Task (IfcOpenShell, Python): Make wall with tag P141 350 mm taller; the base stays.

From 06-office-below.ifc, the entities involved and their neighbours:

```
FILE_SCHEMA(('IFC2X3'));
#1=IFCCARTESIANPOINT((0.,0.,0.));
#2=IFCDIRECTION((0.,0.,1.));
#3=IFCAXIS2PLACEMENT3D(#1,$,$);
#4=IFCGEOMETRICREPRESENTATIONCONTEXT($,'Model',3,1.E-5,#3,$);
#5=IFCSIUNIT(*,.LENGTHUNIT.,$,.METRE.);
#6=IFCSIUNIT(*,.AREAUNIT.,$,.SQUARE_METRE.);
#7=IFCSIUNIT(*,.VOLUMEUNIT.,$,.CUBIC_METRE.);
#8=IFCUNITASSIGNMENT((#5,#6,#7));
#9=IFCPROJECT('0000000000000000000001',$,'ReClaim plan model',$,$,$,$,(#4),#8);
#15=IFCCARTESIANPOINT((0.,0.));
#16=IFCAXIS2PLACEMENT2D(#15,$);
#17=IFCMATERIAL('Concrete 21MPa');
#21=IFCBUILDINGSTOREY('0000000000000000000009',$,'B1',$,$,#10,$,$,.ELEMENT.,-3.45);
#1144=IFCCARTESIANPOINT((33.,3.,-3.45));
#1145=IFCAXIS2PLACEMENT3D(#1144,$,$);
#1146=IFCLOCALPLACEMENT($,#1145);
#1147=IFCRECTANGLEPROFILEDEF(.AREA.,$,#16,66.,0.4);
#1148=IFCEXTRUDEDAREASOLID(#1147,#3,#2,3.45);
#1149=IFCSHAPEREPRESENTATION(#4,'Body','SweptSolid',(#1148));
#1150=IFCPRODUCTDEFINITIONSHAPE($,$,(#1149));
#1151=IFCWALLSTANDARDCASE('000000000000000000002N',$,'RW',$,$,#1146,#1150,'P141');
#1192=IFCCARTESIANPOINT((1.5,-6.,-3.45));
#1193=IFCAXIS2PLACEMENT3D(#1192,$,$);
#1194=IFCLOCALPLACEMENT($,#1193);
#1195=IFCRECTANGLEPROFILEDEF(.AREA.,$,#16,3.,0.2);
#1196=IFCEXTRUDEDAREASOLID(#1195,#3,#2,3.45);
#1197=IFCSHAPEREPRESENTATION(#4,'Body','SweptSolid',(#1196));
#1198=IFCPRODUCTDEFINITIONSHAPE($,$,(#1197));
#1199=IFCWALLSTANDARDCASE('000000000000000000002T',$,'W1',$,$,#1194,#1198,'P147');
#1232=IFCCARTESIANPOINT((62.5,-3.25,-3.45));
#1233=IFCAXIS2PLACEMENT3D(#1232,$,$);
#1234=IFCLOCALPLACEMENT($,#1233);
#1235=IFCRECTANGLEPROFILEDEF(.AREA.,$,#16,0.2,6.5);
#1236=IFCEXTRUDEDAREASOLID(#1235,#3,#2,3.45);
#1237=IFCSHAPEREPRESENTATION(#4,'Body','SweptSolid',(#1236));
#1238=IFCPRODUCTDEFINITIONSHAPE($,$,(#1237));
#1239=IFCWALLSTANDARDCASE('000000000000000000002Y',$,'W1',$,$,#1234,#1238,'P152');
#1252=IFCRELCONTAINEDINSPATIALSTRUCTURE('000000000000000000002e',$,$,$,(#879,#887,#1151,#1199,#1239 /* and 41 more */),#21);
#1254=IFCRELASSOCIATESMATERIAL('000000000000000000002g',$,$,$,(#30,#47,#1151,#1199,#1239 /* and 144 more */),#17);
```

```python
import ifcopenshell
import ifcopenshell.geom
import ifcopenshell.util.shape

model = ifcopenshell.open("06-office-below.ifc")
settings = ifcopenshell.geom.settings()


def volume(element):
    """Net volume in cubic metres, openings subtracted."""
    shape = ifcopenshell.geom.create_shape(settings, element)
    return ifcopenshell.util.shape.get_volume(shape.geometry)


wall = model.by_id(1151)
before = volume(wall)

body = next(r for r in wall.Representation.Representations if r.RepresentationIdentifier == "Body")
solid = body.Items[0]
old_height = solid.Depth
solid.Depth += 0.35
after = volume(wall)

print(f"height {old_height:g} -> {solid.Depth:g}, volume {before:.3f} -> {after:.3f} m3")

model.write("06-office-below_rev.ifc")
```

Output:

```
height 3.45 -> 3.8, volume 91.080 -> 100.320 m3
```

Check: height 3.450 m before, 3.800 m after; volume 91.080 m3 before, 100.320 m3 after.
